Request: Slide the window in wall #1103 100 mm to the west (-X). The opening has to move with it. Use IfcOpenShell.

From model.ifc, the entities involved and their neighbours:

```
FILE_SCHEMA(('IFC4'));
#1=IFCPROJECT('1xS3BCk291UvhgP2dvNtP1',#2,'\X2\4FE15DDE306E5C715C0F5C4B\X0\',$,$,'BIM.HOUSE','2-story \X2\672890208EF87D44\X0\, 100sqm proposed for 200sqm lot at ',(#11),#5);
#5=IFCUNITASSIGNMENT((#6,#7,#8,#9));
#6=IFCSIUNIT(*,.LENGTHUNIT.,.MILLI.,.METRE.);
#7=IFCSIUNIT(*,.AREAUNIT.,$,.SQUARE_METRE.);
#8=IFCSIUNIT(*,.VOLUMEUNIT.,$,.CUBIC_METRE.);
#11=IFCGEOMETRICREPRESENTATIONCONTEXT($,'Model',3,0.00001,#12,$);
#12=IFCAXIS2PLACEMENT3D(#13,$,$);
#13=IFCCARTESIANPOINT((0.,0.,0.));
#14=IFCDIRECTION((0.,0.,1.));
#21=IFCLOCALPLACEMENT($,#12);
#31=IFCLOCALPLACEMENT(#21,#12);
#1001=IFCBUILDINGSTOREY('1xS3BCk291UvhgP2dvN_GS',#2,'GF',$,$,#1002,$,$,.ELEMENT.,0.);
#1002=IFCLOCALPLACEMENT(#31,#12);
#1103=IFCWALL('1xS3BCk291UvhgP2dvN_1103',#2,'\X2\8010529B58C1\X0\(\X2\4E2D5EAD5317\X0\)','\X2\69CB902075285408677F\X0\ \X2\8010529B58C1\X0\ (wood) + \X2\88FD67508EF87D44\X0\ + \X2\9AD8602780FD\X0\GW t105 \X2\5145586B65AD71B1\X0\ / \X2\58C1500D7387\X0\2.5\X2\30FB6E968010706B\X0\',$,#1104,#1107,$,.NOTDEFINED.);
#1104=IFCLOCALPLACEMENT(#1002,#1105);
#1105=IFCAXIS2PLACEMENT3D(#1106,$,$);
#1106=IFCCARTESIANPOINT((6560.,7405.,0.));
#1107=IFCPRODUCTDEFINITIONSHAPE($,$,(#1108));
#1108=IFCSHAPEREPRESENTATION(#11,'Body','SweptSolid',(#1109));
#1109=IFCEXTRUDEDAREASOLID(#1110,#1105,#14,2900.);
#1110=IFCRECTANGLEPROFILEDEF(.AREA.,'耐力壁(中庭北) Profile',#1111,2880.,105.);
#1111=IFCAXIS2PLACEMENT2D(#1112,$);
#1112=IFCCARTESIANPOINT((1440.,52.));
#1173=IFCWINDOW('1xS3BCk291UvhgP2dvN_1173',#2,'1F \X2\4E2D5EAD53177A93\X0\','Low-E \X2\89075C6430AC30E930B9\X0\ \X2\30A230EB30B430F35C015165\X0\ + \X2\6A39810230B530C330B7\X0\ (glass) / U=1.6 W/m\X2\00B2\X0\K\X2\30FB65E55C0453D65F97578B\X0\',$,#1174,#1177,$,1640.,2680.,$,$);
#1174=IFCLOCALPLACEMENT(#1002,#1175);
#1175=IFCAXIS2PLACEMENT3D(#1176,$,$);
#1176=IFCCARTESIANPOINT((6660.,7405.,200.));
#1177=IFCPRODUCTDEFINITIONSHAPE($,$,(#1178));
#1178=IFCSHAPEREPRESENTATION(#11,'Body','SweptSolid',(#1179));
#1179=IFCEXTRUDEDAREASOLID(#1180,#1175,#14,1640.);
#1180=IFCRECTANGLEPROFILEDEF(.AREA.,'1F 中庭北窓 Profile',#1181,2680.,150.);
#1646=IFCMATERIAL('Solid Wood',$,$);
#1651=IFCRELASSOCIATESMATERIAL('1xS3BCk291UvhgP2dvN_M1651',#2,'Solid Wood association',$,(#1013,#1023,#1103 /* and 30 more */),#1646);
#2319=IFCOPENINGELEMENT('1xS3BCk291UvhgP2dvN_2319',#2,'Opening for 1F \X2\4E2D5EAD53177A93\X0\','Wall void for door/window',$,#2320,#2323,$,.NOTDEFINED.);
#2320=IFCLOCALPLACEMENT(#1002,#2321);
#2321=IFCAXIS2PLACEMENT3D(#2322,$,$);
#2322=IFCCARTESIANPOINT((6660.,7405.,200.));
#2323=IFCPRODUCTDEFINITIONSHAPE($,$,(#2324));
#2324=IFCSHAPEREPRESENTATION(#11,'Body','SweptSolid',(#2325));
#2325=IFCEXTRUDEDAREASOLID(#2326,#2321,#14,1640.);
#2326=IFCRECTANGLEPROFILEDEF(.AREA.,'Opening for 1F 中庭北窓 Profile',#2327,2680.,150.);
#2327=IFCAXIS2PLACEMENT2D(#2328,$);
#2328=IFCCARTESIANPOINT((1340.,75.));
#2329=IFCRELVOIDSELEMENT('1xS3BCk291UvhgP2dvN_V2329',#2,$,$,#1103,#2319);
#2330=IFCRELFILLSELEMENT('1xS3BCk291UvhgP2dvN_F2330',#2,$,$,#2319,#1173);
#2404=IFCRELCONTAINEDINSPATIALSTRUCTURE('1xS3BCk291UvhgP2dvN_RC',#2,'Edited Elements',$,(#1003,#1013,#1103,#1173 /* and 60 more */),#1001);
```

```python
import ifcopenshell
import ifcopenshell.api.geometry
import ifcopenshell.util.placement
import ifcopenshell.util.unit

model = ifcopenshell.open("model.ifc")
unit_scale = ifcopenshell.util.unit.calculate_unit_scale(model)

window = model.by_id(1173)
opening = window.FillsVoids[0].RelatingOpeningElement
wall = opening.VoidsElements[0].RelatingBuildingElement

wall_matrix = ifcopenshell.util.placement.get_local_placement(wall.ObjectPlacement)
shift = wall_matrix[:3, 0] * -0.1 / unit_scale
before = ifcopenshell.util.placement.get_local_placement(window.ObjectPlacement)[:3, 3].copy()

# The window is not placed relative to its opening, so move both.
for product in (opening, window):
    matrix = ifcopenshell.util.placement.get_local_placement(product.ObjectPlacement)
    matrix[:3, 3] += shift
    ifcopenshell.api.geometry.edit_object_placement(model, product=product, matrix=matrix, is_si=False)

after = ifcopenshell.util.placement.get_local_placement(window.ObjectPlacement)[:3, 3]
print("window moved by", (after - before).round(3) + 0.0)

model.write("model_updated.ifc")
```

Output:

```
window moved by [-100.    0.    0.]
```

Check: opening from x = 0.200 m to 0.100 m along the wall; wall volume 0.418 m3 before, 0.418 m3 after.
